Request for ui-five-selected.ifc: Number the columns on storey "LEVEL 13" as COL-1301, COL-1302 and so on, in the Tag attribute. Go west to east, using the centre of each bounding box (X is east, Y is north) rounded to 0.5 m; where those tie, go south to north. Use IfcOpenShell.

First a look at what the model holds.

```python
import ifcopenshell
import ifcopenshell.util.element
import ifcopenshell.util.placement

model = ifcopenshell.open("ui-five-selected.ifc")
print(model.schema)
storey = next(s for s in model.by_type("IfcBuildingStorey") if s.Name == "LEVEL 13")
columns = [e for e in ifcopenshell.util.element.get_decomposition(storey) if e.is_a("IfcColumn")]
for e in sorted(columns, key=lambda e: e.id()):
    origin = ifcopenshell.util.placement.get_local_placement(e.ObjectPlacement)[:3, 3]
    print(e.id(), e.Tag, e.Name, origin.round(2) + 0.0, sep=" | ")
```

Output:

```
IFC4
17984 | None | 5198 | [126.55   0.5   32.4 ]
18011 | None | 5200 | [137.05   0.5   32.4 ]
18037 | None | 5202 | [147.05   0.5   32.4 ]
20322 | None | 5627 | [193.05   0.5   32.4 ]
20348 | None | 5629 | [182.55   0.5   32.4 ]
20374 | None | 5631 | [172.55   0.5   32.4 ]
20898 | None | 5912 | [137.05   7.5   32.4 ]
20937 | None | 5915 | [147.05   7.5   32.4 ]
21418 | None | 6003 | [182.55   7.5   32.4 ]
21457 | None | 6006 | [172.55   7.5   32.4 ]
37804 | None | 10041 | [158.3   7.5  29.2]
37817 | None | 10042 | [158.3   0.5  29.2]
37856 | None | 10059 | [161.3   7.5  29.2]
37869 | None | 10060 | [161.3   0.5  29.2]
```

```python
import ifcopenshell
import ifcopenshell.geom
import ifcopenshell.util.element
import ifcopenshell.util.shape

model = ifcopenshell.open("ui-five-selected.ifc")
settings = ifcopenshell.geom.settings()
settings.set("use-world-coords", True)


def centre(element):
    shape = ifcopenshell.geom.create_shape(settings, element)
    return ifcopenshell.util.shape.get_bbox_centroid(shape.geometry)


storey = next(s for s in model.by_type("IfcBuildingStorey") if s.Name == "LEVEL 13")
columns = [e for e in ifcopenshell.util.element.get_decomposition(storey) if e.is_a("IfcColumn")]

# Insertion points can sit at a corner or the storey origin, so sort by the geometry (in metres).
centres = {e: centre(e) for e in columns}
columns.sort(key=lambda e: (round(centres[e][0] / 0.5), centres[e][1]))

for i, e in enumerate(columns, start=1):
    number = f"COL-13{i:02d}"
    e.Tag = number
    print(e.id(), number)

model.write("ui-five-selected_updated.ifc")
```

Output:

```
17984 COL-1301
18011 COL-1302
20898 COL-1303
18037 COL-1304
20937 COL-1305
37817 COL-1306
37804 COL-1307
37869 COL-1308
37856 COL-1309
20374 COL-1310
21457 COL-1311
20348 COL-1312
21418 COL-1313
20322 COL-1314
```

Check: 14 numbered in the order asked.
